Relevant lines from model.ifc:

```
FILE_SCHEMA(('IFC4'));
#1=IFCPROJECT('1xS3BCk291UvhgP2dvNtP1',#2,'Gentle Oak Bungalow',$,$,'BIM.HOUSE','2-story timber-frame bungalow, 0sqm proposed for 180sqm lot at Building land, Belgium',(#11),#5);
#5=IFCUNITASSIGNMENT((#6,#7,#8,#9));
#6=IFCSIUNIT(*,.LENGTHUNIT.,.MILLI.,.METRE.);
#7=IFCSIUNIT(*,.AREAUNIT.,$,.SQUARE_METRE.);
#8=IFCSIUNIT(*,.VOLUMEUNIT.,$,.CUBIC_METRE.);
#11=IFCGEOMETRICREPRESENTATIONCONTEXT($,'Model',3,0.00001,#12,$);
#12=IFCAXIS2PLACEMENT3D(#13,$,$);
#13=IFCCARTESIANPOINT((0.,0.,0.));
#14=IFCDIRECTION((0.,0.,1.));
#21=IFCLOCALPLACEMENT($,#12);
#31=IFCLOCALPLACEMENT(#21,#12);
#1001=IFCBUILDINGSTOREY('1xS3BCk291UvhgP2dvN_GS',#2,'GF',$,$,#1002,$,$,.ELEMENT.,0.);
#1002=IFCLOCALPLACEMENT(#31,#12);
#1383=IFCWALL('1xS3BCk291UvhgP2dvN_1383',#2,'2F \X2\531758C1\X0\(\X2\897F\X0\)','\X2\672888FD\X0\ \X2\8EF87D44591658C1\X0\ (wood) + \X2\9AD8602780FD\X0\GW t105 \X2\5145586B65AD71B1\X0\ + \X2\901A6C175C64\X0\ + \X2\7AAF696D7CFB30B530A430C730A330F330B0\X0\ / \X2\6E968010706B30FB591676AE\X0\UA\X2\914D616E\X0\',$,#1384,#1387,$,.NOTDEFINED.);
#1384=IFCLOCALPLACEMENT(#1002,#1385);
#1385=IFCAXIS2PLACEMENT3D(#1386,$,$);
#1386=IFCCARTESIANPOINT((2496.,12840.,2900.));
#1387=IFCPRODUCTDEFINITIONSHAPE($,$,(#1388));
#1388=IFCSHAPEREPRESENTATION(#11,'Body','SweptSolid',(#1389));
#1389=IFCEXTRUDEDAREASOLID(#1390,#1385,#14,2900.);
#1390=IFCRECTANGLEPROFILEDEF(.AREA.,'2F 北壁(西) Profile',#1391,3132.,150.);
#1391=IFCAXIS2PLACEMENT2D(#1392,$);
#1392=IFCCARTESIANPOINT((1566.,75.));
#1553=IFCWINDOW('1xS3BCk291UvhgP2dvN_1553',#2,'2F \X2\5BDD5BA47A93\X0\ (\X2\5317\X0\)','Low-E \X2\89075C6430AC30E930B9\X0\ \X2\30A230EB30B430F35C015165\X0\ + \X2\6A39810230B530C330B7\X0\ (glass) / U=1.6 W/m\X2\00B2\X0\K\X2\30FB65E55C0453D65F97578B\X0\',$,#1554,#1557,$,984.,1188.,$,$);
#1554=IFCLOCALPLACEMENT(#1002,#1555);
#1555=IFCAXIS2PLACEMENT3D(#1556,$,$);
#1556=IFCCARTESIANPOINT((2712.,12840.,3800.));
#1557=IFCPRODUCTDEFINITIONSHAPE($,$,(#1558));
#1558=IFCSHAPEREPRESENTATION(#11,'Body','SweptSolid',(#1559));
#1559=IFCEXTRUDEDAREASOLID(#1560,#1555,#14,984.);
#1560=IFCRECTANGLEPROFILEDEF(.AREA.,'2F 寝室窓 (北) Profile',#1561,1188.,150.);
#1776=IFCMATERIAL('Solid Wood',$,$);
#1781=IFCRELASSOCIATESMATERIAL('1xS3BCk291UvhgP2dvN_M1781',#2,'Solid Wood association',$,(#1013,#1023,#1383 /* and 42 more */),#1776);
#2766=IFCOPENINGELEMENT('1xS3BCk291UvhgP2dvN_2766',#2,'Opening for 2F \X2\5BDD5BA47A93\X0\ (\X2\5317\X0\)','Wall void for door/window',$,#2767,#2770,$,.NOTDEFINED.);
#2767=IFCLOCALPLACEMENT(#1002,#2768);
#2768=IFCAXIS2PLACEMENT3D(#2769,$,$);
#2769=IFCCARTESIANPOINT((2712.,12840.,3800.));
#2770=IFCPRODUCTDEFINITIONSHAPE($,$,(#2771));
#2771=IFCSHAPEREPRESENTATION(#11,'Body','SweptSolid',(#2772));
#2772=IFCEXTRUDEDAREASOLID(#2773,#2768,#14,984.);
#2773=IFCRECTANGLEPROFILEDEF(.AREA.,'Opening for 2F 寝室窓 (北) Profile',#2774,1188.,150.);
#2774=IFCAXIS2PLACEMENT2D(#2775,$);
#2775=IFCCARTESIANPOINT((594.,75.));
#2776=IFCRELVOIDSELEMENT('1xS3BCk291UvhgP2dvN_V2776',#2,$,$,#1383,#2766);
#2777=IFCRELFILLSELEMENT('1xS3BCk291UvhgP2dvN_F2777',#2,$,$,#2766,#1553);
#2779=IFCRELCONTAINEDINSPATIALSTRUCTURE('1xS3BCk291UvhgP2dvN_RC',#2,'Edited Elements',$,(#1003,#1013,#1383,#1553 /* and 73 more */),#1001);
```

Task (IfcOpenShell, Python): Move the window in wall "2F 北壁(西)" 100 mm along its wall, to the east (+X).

```python
import ifcopenshell
import ifcopenshell.api.geometry
import ifcopenshell.util.placement

model = ifcopenshell.open("model.ifc")

window = model.by_guid("1xS3BCk291UvhgP2dvN_1553")
opening = window.FillsVoids[0].RelatingOpeningElement
wall = opening.VoidsElements[0].RelatingBuildingElement

wall_matrix = ifcopenshell.util.placement.get_local_placement(wall.ObjectPlacement)
shift = wall_matrix[:3, 0] * 100.0
before = ifcopenshell.util.placement.get_local_placement(window.ObjectPlacement)[:3, 3].copy()

# The window is not placed relative to its opening, so move both.
for product in (opening, window):
    matrix = ifcopenshell.util.placement.get_local_placement(product.ObjectPlacement)
    matrix[:3, 3] += shift
    ifcopenshell.api.geometry.edit_object_placement(model, product=product, matrix=matrix, is_si=False)

after = ifcopenshell.util.placement.get_local_placement(window.ObjectPlacement)[:3, 3]
print("window moved by", (after - before).round(3) + 0.0)

model.write("model_edited.ifc")
```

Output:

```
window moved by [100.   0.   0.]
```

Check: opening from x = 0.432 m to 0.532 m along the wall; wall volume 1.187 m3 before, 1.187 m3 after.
